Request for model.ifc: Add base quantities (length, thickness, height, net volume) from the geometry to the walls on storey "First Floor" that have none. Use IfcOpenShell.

First a look at what the model holds.

```python
import ifcopenshell
import ifcopenshell.util.element
import ifcopenshell.util.unit

model = ifcopenshell.open("model.ifc")
print(model.schema)
for unit_type in ("LENGTHUNIT", "AREAUNIT", "VOLUMEUNIT"):
    print(unit_type, ifcopenshell.util.unit.calculate_unit_scale(model, unit_type))
storey = next(s for s in model.by_type("IfcBuildingStorey") if s.Name == "First Floor")
walls = [e for e in ifcopenshell.util.element.get_decomposition(storey) if e.is_a("IfcWall")]
for e in sorted(walls, key=lambda e: e.id()):
    print(e.id(), e.is_a(), e.Name, list(ifcopenshell.util.element.get_psets(e, qtos_only=True)), sep=" | ")
```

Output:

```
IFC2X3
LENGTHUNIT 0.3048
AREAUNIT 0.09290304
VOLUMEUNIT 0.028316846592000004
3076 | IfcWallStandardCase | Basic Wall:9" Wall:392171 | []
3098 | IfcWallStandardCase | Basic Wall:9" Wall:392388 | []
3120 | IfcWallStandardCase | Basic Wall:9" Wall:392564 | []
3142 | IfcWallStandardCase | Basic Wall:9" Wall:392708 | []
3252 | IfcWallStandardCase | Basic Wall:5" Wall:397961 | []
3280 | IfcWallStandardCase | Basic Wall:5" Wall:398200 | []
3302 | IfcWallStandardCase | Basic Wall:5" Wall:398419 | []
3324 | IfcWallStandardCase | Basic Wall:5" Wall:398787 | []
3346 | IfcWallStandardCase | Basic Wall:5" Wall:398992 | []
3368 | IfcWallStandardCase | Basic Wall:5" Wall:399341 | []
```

```python
import ifcopenshell
import ifcopenshell.api.pset
import ifcopenshell.geom
import ifcopenshell.util.element
import ifcopenshell.util.shape
import ifcopenshell.util.unit

model = ifcopenshell.open("model.ifc")
unit_scale = ifcopenshell.util.unit.calculate_unit_scale(model)
volume_scale = ifcopenshell.util.unit.calculate_unit_scale(model, "VOLUMEUNIT")
settings = ifcopenshell.geom.settings()

storey = next(s for s in model.by_type("IfcBuildingStorey") if s.Name == "First Floor")
walls = [e for e in ifcopenshell.util.element.get_decomposition(storey) if e.is_a("IfcWall")]

for e in sorted(walls, key=lambda e: e.id()):
    if ifcopenshell.util.element.get_psets(e, qtos_only=True, should_inherit=False):
        continue
    # Geometry comes back in metres, in the element's own axes.
    shape = ifcopenshell.geom.create_shape(settings, e)
    values = {
        "Length": ifcopenshell.util.shape.get_x(shape.geometry) / unit_scale,
        "Width": ifcopenshell.util.shape.get_y(shape.geometry) / unit_scale,
        "Height": ifcopenshell.util.shape.get_z(shape.geometry) / unit_scale,
        "NetVolume": ifcopenshell.util.shape.get_volume(shape.geometry) / volume_scale,
    }
    qto = ifcopenshell.api.pset.add_qto(model, product=e, name="BaseQuantities")
    ifcopenshell.api.pset.edit_qto(model, qto=qto, properties=values)
    print(e.id(), {k: round(v, 3) for k, v in values.items()})

model.write("model-out.ifc")
```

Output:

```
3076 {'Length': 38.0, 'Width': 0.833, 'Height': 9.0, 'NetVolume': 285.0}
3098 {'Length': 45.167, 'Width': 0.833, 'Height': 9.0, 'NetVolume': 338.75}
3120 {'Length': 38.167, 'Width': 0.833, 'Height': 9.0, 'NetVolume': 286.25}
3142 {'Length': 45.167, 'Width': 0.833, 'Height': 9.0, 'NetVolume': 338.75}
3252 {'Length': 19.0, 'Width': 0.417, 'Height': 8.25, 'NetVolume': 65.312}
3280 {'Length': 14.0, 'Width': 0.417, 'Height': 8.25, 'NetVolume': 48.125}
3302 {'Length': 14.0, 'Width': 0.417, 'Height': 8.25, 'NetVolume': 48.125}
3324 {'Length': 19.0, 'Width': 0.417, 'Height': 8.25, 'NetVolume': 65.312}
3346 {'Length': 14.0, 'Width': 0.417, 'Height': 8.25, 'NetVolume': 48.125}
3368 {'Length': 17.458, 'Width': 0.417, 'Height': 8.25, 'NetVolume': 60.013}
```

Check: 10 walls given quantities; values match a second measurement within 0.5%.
